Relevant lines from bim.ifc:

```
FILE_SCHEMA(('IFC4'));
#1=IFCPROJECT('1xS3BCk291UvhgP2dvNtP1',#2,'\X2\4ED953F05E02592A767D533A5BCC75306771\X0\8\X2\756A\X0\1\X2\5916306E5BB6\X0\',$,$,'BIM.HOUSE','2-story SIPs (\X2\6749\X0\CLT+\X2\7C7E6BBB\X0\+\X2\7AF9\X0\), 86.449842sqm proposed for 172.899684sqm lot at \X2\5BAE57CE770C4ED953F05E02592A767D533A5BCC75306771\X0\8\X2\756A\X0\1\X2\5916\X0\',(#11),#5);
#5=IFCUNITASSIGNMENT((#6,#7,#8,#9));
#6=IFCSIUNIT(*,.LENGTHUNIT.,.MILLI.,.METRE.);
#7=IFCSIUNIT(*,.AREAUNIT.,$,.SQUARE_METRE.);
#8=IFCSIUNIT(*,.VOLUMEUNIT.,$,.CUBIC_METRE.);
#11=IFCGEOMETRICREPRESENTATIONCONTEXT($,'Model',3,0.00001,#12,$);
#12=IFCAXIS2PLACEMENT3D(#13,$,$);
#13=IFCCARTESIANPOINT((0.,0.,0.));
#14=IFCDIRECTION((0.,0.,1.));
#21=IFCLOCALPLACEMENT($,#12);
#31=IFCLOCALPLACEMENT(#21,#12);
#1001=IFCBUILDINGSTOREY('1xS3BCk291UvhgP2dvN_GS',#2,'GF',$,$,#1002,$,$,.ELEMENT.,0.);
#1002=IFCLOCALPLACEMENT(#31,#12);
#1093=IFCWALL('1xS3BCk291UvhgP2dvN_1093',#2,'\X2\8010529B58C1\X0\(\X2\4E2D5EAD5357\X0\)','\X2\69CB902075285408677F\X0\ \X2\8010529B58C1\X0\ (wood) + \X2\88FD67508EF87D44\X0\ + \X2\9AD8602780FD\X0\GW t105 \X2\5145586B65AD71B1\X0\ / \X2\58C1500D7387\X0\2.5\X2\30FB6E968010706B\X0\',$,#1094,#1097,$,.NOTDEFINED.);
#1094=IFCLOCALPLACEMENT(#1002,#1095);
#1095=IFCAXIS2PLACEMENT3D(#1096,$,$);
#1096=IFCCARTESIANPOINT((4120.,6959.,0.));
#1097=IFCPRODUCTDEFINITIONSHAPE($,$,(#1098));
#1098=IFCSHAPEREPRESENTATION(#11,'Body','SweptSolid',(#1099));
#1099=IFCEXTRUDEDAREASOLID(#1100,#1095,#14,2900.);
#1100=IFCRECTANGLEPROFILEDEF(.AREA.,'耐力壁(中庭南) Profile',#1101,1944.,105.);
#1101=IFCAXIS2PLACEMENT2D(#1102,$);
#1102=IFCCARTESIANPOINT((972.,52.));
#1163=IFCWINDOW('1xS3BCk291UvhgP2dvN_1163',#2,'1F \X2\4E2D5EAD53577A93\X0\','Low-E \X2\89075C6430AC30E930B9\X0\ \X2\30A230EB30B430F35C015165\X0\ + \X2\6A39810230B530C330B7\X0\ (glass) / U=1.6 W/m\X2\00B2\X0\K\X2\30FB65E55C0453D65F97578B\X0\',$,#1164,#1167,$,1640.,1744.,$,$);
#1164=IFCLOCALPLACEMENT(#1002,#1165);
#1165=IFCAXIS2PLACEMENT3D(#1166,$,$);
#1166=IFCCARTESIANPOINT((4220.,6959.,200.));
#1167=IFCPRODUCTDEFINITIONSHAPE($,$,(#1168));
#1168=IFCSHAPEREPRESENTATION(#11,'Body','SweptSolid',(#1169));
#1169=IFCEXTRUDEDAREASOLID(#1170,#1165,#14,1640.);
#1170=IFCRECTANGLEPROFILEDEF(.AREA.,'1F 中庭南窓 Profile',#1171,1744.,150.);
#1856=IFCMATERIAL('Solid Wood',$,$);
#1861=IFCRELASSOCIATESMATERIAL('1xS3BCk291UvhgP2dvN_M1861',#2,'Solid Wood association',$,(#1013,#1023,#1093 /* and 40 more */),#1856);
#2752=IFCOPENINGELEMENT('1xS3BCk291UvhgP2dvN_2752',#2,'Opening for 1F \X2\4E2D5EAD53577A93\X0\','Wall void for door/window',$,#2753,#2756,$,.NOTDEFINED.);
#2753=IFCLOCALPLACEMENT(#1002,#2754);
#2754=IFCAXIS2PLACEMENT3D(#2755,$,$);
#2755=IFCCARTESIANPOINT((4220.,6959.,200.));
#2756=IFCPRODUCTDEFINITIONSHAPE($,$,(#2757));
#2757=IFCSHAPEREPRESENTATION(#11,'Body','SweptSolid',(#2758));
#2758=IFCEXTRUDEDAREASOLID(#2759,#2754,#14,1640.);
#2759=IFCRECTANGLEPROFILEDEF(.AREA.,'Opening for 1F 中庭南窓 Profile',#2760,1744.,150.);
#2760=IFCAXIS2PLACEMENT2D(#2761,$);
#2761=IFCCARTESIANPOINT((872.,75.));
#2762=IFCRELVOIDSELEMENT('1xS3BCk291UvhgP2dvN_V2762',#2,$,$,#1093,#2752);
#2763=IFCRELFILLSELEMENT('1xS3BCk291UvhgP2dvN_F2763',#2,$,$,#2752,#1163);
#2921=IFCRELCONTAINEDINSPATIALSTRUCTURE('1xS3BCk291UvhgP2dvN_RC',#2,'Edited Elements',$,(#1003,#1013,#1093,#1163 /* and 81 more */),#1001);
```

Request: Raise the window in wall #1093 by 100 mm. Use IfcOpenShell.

```python
import numpy as np
import ifcopenshell
import ifcopenshell.api.geometry
import ifcopenshell.util.placement
import ifcopenshell.util.unit

model = ifcopenshell.open("bim.ifc")
unit_scale = ifcopenshell.util.unit.calculate_unit_scale(model)

window = model.by_id(1163)
opening = window.FillsVoids[0].RelatingOpeningElement
dz = 0.1 / unit_scale

shift = np.array([0.0, 0.0, dz])
# The window is not placed relative to its opening, so move both.
for product in (opening, window):
    matrix = ifcopenshell.util.placement.get_local_placement(product.ObjectPlacement)
    matrix[:3, 3] += shift
    ifcopenshell.api.geometry.edit_object_placement(model, product=product, matrix=matrix, is_si=False)

print(f"moved by {dz * unit_scale:+.3f} m")

model.write("bim_updated.ifc")
```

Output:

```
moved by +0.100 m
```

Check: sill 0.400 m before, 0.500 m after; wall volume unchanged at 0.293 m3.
